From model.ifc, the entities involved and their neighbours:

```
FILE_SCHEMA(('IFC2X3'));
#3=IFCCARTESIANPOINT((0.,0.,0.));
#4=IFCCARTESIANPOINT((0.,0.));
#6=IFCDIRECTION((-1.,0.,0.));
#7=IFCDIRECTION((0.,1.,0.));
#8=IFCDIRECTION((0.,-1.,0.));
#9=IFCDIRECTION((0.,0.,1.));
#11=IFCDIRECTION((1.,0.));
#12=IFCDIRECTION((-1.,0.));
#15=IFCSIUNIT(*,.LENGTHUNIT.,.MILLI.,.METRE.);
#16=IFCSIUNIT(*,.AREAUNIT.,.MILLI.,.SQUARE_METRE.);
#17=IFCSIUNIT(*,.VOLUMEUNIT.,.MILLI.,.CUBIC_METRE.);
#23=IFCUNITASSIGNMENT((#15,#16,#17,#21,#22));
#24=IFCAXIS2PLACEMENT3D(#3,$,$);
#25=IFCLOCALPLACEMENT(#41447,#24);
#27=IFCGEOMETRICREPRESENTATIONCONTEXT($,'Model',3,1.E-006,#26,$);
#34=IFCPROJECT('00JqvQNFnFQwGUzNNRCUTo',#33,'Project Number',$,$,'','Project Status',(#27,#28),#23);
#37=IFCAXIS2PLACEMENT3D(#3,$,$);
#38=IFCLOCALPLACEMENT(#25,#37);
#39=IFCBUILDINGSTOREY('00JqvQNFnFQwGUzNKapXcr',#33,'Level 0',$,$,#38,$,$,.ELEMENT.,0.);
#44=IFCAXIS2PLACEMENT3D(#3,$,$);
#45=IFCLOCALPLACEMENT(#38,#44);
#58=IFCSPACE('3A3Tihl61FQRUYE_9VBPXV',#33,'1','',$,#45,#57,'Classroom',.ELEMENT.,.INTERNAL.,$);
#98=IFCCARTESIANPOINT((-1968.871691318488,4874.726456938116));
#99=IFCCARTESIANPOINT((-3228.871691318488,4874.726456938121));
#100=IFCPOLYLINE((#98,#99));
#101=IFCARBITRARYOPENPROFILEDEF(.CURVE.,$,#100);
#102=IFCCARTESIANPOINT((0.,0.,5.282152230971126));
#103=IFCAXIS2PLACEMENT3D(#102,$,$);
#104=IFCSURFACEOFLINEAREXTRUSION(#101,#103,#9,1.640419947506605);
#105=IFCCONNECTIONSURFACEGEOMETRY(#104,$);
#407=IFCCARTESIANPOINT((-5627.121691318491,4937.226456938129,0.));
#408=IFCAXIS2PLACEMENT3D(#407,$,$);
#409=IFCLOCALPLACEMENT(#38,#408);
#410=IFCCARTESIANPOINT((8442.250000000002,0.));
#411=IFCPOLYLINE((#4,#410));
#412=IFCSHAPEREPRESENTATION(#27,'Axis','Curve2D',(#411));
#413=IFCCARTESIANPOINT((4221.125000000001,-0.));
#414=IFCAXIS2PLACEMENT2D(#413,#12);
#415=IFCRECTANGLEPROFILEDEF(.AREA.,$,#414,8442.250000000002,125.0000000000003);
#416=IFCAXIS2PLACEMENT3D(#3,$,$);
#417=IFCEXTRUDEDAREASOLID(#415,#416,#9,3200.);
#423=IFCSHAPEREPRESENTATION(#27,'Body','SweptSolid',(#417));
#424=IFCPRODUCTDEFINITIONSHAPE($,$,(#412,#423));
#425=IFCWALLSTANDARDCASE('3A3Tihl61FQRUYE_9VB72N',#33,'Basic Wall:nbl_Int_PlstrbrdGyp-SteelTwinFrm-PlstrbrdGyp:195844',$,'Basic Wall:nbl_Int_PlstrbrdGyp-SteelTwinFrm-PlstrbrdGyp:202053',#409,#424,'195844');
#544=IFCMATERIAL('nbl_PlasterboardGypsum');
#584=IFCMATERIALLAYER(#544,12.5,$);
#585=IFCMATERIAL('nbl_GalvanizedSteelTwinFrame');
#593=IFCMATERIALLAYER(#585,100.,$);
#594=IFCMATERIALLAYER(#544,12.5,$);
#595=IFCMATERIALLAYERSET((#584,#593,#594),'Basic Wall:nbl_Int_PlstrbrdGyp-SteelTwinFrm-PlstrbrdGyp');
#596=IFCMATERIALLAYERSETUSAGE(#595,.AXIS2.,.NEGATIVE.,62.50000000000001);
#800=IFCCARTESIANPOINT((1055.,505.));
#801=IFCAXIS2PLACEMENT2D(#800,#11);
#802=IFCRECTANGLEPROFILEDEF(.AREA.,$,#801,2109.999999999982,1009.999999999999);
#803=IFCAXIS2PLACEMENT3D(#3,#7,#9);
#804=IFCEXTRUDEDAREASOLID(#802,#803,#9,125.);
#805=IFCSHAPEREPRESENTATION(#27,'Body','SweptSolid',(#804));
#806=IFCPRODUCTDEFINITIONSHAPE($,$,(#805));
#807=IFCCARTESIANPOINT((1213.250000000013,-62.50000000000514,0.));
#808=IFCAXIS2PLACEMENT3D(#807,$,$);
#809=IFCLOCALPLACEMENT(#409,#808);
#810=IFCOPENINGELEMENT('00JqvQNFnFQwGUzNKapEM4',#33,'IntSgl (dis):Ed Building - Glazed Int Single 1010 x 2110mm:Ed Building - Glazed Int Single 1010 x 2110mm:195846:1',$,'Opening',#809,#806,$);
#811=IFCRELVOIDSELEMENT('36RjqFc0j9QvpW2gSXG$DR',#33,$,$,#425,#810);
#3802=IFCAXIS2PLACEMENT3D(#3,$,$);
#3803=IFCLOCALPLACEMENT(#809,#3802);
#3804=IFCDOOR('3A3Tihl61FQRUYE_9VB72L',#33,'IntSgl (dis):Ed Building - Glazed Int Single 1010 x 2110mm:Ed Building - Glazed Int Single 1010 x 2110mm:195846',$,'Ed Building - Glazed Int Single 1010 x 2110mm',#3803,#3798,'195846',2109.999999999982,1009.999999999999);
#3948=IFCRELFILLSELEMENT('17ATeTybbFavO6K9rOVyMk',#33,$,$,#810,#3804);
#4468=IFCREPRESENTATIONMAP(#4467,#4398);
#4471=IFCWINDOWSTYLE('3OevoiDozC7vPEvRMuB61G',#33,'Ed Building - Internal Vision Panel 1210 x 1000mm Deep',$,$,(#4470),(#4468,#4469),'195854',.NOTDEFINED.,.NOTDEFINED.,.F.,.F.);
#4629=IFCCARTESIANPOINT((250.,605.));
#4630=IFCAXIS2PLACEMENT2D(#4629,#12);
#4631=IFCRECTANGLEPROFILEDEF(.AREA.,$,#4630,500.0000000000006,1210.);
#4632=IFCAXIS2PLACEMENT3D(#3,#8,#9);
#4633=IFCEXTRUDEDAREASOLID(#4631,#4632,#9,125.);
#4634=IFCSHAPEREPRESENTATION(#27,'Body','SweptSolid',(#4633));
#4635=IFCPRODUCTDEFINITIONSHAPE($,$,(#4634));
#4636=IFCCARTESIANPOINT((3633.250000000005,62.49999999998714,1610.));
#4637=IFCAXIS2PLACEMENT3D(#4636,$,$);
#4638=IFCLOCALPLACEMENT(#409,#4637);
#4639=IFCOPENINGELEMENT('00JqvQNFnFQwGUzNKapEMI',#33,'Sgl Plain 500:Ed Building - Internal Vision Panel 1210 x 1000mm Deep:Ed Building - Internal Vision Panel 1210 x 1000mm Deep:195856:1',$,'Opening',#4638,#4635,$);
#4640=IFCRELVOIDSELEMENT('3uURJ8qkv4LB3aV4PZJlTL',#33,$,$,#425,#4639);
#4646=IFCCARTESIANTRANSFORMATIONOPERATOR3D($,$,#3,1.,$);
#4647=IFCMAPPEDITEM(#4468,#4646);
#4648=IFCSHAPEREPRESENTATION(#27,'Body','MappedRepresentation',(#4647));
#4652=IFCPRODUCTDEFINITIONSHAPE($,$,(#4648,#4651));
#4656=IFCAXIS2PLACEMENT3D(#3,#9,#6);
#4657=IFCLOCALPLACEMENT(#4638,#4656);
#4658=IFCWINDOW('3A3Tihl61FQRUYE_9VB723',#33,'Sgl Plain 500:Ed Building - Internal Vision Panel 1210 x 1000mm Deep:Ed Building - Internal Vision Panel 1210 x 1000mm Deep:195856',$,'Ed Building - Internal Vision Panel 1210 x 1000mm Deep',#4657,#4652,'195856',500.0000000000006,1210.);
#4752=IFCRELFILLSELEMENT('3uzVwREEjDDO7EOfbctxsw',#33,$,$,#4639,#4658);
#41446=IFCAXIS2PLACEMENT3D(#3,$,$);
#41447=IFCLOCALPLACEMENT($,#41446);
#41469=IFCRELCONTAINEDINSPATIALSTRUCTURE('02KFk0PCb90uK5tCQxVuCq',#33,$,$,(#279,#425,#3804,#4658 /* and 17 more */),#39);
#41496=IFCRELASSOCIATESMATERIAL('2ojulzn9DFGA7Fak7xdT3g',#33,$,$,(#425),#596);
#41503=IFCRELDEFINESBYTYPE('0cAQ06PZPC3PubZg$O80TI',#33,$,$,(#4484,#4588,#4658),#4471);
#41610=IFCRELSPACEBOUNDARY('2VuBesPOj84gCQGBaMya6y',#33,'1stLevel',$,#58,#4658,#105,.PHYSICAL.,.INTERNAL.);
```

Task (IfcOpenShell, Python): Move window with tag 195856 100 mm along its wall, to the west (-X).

```python
import numpy as np
import ifcopenshell
import ifcopenshell.api.geometry
import ifcopenshell.util.placement
import ifcopenshell.util.unit

model = ifcopenshell.open("model.ifc")
unit_scale = ifcopenshell.util.unit.calculate_unit_scale(model)

window = model.by_id(4658)
opening = window.FillsVoids[0].RelatingOpeningElement
wall = opening.VoidsElements[0].RelatingBuildingElement

wall_matrix = ifcopenshell.util.placement.get_local_placement(wall.ObjectPlacement)
shift = wall_matrix[:3, 0] * -0.1 / unit_scale
before = ifcopenshell.util.placement.get_local_placement(window.ObjectPlacement)[:3, 3].copy()

# The window is placed relative to its opening, so it follows when the opening moves.
matrix = ifcopenshell.util.placement.get_local_placement(opening.ObjectPlacement)
matrix[:3, 3] += shift
ifcopenshell.api.geometry.edit_object_placement(
    model, product=opening, matrix=matrix, is_si=False, should_transform_children=True
)

# Space boundary surfaces are stored in each space's coordinates; move them too.
for rel in window.ProvidesBoundaries:
    if not rel.ConnectionGeometry:
        continue
    surface = rel.ConnectionGeometry.SurfaceOnRelatingElement
    space_matrix = ifcopenshell.util.placement.get_local_placement(rel.RelatingSpace.ObjectPlacement)
    point = np.array(surface.Position.Location.Coordinates) + space_matrix[:3, :3].T @ shift
    surface.Position = model.createIfcAxis2Placement3D(
        model.createIfcCartesianPoint(point.tolist()), surface.Position.Axis, surface.Position.RefDirection
    )

after = ifcopenshell.util.placement.get_local_placement(window.ObjectPlacement)[:3, 3]
print("window moved by", (after - before).round(3) + 0.0)

model.write("model_updated.ifc")
```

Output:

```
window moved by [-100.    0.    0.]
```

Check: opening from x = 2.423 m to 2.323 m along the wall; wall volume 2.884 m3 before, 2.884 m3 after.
